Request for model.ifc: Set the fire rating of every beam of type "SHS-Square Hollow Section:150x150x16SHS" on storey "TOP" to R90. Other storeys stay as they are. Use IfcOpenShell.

First a look at what the model holds.

```python
import ifcopenshell
import ifcopenshell.util.element

model = ifcopenshell.open("model.ifc")
print(model.schema)
storey = next(s for s in model.by_type("IfcBuildingStorey") if s.Name == "TOP")
beams = [e for e in ifcopenshell.util.element.get_decomposition(storey) if e.is_a("IfcBeam")]
seen = {}
for e in beams:
    element_type = ifcopenshell.util.element.get_type(e)
    key = (element_type.Name if element_type != e and element_type else None, ifcopenshell.util.element.get_pset(e, "Pset_BeamCommon", "FireRating"))
    seen[key] = seen.get(key, 0) + 1
for (name, value), count in sorted(seen.items(), key=str):
    print(count, "x", name, "|", value)
```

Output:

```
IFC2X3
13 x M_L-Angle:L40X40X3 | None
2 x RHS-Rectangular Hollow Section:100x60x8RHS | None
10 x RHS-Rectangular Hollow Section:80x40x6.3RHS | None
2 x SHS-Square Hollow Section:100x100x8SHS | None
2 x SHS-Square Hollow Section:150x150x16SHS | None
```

```python
import ifcopenshell
import ifcopenshell.api.pset
import ifcopenshell.util.element

model = ifcopenshell.open("model.ifc")

storey = next(s for s in model.by_type("IfcBuildingStorey") if s.Name == "TOP")
beams = [e for e in ifcopenshell.util.element.get_decomposition(storey) if e.is_a("IfcBeam")]

count = 0
for e in beams:
    element_type = ifcopenshell.util.element.get_type(e)
    if element_type in (None, e) or element_type.Name != "SHS-Square Hollow Section:150x150x16SHS":
        continue
    # add_pset returns the element's existing set when there is one.
    pset = ifcopenshell.api.pset.add_pset(model, product=e, name="Pset_BeamCommon")
    ifcopenshell.api.pset.edit_pset(model, pset=pset, properties={"FireRating": "R90"})
    count += 1

print(count, "beams updated")

model.write("model-out.ifc")
```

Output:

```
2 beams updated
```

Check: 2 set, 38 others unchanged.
